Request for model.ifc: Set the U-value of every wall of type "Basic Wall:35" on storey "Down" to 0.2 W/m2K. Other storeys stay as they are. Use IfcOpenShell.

First a look at what the model holds.

```python
import ifcopenshell
import ifcopenshell.util.element

model = ifcopenshell.open("model.ifc")
print(model.schema)
storey = next(s for s in model.by_type("IfcBuildingStorey") if s.Name == "Down")
walls = [e for e in ifcopenshell.util.element.get_decomposition(storey) if e.is_a("IfcWall")]
seen = {}
for e in walls:
    element_type = ifcopenshell.util.element.get_type(e)
    key = (element_type.Name if element_type != e and element_type else None, ifcopenshell.util.element.get_pset(e, "Pset_WallCommon", "ThermalTransmittance"))
    seen[key] = seen.get(key, 0) + 1
for (name, value), count in sorted(seen.items(), key=str):
    print(count, "x", name, "|", value)
```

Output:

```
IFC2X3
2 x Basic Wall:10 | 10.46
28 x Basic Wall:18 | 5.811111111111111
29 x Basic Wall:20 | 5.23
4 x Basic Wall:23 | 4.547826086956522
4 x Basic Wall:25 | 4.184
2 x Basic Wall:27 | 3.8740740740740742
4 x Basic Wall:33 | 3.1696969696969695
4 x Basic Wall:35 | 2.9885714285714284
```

```python
import ifcopenshell
import ifcopenshell.api.pset
import ifcopenshell.util.element

model = ifcopenshell.open("model.ifc")

storey = next(s for s in model.by_type("IfcBuildingStorey") if s.Name == "Down")
walls = [e for e in ifcopenshell.util.element.get_decomposition(storey) if e.is_a("IfcWall")]

count = 0
for e in walls:
    element_type = ifcopenshell.util.element.get_type(e)
    if element_type in (None, e) or element_type.Name != "Basic Wall:35":
        continue
    # add_pset returns the element's existing set when there is one.
    pset = ifcopenshell.api.pset.add_pset(model, product=e, name="Pset_WallCommon")
    ifcopenshell.api.pset.edit_pset(model, pset=pset, properties={"ThermalTransmittance": 0.2})
    count += 1

print(count, "walls updated")

model.write("model-out.ifc")
```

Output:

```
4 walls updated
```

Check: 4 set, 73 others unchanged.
